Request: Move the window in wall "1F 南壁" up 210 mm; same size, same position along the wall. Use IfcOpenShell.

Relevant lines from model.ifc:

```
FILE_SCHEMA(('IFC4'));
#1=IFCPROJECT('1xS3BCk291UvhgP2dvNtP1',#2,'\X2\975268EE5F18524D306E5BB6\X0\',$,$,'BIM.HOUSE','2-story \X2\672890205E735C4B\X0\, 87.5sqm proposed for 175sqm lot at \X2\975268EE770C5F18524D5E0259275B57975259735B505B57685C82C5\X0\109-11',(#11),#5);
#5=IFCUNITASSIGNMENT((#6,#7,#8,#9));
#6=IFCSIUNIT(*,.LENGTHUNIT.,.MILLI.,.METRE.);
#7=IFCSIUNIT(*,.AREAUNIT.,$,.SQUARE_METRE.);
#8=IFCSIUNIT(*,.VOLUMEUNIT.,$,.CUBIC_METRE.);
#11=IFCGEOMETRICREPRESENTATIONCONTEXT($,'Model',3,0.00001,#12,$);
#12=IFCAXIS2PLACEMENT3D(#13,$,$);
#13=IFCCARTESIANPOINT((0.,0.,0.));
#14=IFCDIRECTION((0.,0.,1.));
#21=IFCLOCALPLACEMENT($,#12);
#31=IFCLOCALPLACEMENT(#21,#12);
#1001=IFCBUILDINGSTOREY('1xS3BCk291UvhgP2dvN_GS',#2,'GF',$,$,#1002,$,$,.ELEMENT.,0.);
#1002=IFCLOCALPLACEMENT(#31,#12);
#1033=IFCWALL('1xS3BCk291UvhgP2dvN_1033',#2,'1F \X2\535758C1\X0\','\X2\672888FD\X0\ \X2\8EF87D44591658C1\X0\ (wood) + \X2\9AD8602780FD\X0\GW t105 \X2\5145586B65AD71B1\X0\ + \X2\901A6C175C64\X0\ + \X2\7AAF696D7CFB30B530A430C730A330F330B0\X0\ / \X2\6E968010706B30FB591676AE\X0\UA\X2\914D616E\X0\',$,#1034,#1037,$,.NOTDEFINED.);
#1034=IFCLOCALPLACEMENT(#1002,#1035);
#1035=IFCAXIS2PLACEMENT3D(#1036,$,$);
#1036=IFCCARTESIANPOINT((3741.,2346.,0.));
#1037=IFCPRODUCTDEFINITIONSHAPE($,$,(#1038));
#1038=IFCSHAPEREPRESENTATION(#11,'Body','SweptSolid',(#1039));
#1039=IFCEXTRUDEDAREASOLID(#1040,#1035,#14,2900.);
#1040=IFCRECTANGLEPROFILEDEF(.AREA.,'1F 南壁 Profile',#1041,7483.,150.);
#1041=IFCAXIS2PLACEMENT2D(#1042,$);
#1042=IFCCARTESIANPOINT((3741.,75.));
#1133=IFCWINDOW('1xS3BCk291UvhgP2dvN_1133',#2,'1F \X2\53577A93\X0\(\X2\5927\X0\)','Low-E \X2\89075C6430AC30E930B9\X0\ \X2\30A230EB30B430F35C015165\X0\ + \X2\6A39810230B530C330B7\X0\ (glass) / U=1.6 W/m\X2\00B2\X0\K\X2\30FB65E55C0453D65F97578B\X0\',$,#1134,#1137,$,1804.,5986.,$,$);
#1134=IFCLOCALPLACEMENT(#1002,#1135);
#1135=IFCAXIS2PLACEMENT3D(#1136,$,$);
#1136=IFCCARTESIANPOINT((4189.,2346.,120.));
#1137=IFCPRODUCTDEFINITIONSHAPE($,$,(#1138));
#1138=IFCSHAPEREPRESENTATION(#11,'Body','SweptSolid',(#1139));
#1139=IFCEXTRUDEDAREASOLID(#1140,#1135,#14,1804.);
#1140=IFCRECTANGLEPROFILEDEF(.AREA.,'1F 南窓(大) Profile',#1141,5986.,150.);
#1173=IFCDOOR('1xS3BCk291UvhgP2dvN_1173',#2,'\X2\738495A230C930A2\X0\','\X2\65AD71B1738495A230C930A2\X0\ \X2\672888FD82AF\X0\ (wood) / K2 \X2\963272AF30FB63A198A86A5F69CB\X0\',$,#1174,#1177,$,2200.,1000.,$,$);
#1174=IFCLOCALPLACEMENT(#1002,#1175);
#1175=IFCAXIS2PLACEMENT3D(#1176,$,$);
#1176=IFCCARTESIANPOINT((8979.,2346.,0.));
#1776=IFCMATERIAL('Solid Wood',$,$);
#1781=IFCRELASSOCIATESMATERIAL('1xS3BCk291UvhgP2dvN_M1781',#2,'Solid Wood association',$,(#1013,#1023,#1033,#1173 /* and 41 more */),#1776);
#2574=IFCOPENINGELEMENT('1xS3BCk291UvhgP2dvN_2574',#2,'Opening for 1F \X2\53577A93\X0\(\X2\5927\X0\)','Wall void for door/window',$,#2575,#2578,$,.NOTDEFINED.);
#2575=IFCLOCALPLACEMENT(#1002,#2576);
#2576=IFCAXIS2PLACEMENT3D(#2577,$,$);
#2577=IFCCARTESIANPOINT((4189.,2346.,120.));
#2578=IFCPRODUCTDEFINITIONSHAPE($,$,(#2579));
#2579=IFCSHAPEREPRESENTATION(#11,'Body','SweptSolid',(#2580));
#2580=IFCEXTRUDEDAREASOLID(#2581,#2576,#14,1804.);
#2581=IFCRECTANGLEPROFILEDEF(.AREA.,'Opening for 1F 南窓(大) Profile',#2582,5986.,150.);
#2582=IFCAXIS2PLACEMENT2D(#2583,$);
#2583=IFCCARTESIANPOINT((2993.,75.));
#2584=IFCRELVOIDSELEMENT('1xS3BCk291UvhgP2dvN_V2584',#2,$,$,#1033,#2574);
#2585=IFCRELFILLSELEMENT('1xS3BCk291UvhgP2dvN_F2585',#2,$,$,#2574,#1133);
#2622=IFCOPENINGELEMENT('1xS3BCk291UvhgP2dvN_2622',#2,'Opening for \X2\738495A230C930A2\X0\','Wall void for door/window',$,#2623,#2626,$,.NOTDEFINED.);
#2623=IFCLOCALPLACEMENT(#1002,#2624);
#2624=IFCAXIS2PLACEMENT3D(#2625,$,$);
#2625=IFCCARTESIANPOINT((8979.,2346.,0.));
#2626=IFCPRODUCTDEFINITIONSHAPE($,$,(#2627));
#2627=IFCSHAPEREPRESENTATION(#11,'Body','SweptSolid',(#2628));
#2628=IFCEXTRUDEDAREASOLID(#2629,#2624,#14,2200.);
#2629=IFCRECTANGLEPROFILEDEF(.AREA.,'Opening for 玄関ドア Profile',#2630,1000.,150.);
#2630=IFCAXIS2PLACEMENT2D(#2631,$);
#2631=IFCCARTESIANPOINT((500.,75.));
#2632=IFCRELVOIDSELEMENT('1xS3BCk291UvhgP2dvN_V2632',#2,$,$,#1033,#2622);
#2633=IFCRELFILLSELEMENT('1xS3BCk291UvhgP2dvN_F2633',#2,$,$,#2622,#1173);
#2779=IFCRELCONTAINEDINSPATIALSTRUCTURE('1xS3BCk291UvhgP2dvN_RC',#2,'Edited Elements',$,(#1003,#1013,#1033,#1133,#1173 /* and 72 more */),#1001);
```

```python
import numpy as np
import ifcopenshell
import ifcopenshell.api.geometry
import ifcopenshell.util.placement
import ifcopenshell.util.unit

model = ifcopenshell.open("model.ifc")
unit_scale = ifcopenshell.util.unit.calculate_unit_scale(model)

window = model.by_guid("1xS3BCk291UvhgP2dvN_1133")
opening = window.FillsVoids[0].RelatingOpeningElement
dz = 0.21 / unit_scale

shift = np.array([0.0, 0.0, dz])
# The window is not placed relative to its opening, so move both.
for product in (opening, window):
    matrix = ifcopenshell.util.placement.get_local_placement(product.ObjectPlacement)
    matrix[:3, 3] += shift
    ifcopenshell.api.geometry.edit_object_placement(model, product=product, matrix=matrix, is_si=False)

print(f"moved by {dz * unit_scale:+.3f} m")

model.write("model_edited.ifc")
```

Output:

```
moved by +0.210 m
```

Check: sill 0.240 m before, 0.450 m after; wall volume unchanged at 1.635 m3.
